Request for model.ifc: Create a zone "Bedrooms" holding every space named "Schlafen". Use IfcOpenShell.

First a look at what the model holds.

```python
import ifcopenshell

model = ifcopenshell.open("model.ifc")
print(model.schema)
seen = {}
for space in model.by_type("IfcSpace"):
    seen[space.LongName] = seen.get(space.LongName, 0) + 1
for name, count in sorted(seen.items(), key=str):
    print(count, "x", name)
print("zones:", [z.Name for z in model.by_type("IfcZone")][:20])
```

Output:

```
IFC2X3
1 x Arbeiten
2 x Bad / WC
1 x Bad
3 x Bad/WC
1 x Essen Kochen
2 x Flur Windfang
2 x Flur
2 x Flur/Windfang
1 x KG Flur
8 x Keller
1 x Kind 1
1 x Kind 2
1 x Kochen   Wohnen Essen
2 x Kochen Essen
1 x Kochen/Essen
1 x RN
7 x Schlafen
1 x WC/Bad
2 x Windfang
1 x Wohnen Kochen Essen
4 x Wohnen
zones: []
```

```python
import ifcopenshell
import ifcopenshell.api.group
import ifcopenshell.api.root

model = ifcopenshell.open("model.ifc")

names = {"Schlafen"}
spaces = [s for s in model.by_type("IfcSpace") if s.LongName in names]

zone = ifcopenshell.api.root.create_entity(model, ifc_class="IfcZone", name="Bedrooms")
ifcopenshell.api.group.assign_group(model, products=spaces, group=zone)
print(len(spaces), "spaces in", zone.Name)

model.write("model-out.ifc")
```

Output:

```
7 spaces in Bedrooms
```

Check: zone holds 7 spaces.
